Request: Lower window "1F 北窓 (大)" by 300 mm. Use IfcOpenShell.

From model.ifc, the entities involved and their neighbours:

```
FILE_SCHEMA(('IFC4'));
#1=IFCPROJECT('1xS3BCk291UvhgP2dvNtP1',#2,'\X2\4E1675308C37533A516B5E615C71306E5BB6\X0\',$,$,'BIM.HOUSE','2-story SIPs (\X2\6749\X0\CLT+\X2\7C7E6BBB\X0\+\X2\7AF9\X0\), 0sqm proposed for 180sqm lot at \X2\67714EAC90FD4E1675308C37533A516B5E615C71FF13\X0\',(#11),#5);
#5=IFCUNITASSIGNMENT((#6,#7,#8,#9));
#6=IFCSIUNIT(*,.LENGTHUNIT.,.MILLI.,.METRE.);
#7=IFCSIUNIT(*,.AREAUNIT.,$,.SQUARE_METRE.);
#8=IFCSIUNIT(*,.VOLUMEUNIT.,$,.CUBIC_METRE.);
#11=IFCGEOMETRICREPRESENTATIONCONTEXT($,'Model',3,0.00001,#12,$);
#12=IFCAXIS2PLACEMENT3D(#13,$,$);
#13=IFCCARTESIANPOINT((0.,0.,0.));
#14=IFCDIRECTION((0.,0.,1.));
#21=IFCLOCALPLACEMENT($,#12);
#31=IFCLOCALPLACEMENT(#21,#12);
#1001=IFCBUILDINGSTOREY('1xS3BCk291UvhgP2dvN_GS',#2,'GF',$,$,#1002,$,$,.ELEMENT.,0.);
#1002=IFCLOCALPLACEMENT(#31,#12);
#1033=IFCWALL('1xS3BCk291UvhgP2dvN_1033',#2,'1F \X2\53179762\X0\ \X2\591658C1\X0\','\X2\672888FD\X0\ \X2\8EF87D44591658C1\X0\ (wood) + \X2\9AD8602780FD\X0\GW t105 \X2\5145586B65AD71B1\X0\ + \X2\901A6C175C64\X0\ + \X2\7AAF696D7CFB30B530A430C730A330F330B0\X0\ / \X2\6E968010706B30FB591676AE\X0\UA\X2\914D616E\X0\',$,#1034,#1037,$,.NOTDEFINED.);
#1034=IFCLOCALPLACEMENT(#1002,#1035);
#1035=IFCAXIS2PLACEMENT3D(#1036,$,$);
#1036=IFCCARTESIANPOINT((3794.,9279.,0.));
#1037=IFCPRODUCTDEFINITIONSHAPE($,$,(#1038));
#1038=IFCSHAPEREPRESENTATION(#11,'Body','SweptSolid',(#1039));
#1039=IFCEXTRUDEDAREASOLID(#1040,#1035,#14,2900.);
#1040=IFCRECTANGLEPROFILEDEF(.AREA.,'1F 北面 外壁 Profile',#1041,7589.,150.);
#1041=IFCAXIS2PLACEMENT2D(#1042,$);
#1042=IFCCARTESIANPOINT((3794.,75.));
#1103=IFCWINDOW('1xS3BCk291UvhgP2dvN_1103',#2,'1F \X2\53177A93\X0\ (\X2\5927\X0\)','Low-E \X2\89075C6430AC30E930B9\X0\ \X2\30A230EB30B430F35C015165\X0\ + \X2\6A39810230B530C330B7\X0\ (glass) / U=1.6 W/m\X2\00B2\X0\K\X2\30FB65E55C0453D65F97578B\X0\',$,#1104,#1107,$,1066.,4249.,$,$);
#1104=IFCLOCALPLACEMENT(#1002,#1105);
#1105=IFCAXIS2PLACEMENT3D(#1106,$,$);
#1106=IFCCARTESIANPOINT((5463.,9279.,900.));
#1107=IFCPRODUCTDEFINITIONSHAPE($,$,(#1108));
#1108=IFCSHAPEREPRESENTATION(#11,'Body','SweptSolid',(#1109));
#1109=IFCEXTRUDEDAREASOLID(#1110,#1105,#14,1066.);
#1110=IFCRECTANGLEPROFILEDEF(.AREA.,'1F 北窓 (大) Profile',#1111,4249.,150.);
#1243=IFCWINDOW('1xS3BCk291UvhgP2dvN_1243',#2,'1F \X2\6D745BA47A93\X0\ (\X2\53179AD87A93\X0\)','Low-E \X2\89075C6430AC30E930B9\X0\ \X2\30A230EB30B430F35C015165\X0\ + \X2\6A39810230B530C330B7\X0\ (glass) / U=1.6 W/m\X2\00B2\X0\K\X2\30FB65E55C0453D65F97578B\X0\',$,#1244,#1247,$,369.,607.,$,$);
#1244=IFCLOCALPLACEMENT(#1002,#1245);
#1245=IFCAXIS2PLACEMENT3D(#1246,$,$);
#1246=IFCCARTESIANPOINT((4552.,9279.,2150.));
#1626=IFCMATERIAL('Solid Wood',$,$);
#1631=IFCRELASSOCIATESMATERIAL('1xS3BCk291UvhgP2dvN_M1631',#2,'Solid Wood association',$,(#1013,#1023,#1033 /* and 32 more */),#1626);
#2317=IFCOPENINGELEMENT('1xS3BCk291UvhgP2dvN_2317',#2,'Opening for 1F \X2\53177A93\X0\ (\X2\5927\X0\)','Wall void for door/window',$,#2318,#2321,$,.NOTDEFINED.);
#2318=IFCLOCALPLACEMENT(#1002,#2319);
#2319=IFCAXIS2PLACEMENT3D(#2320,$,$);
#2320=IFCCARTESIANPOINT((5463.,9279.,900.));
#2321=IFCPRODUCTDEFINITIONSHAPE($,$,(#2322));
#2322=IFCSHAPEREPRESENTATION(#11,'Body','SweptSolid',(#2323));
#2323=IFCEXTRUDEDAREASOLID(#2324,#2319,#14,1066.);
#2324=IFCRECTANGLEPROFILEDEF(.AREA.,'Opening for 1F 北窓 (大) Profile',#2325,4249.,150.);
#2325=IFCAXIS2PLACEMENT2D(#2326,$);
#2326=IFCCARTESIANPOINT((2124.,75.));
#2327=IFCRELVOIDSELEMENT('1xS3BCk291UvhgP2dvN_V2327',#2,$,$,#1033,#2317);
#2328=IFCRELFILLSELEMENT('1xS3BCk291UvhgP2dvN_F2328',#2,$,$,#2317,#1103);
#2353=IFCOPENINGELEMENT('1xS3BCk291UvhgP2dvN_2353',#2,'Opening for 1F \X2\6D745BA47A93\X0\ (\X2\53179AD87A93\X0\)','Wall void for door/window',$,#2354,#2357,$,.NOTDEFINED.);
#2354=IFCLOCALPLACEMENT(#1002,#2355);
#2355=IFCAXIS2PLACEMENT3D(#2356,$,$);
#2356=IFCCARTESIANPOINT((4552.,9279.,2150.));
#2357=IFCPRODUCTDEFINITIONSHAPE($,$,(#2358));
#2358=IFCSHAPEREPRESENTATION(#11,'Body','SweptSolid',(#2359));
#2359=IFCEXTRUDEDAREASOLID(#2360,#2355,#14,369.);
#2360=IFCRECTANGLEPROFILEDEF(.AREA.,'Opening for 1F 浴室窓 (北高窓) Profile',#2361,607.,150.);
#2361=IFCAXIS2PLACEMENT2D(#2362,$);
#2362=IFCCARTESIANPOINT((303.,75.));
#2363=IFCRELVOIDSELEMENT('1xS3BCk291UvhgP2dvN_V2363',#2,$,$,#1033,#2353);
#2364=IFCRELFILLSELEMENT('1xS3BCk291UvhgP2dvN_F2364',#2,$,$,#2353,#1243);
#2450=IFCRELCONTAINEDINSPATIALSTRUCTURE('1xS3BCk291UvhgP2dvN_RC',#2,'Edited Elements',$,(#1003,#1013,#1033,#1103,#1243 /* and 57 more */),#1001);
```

```python
import numpy as np
import ifcopenshell
import ifcopenshell.api.geometry
import ifcopenshell.util.placement
import ifcopenshell.util.unit

model = ifcopenshell.open("model.ifc")
unit_scale = ifcopenshell.util.unit.calculate_unit_scale(model)

window = model.by_id(1103)
opening = window.FillsVoids[0].RelatingOpeningElement
dz = -0.3 / unit_scale

shift = np.array([0.0, 0.0, dz])
# The window is not placed relative to its opening, so move both.
for product in (opening, window):
    matrix = ifcopenshell.util.placement.get_local_placement(product.ObjectPlacement)
    matrix[:3, 3] += shift
    ifcopenshell.api.geometry.edit_object_placement(model, product=product, matrix=matrix, is_si=False)

print(f"moved by {dz * unit_scale:+.3f} m")

model.write("model_updated.ifc")
```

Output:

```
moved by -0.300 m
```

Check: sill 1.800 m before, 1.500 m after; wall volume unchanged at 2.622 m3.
